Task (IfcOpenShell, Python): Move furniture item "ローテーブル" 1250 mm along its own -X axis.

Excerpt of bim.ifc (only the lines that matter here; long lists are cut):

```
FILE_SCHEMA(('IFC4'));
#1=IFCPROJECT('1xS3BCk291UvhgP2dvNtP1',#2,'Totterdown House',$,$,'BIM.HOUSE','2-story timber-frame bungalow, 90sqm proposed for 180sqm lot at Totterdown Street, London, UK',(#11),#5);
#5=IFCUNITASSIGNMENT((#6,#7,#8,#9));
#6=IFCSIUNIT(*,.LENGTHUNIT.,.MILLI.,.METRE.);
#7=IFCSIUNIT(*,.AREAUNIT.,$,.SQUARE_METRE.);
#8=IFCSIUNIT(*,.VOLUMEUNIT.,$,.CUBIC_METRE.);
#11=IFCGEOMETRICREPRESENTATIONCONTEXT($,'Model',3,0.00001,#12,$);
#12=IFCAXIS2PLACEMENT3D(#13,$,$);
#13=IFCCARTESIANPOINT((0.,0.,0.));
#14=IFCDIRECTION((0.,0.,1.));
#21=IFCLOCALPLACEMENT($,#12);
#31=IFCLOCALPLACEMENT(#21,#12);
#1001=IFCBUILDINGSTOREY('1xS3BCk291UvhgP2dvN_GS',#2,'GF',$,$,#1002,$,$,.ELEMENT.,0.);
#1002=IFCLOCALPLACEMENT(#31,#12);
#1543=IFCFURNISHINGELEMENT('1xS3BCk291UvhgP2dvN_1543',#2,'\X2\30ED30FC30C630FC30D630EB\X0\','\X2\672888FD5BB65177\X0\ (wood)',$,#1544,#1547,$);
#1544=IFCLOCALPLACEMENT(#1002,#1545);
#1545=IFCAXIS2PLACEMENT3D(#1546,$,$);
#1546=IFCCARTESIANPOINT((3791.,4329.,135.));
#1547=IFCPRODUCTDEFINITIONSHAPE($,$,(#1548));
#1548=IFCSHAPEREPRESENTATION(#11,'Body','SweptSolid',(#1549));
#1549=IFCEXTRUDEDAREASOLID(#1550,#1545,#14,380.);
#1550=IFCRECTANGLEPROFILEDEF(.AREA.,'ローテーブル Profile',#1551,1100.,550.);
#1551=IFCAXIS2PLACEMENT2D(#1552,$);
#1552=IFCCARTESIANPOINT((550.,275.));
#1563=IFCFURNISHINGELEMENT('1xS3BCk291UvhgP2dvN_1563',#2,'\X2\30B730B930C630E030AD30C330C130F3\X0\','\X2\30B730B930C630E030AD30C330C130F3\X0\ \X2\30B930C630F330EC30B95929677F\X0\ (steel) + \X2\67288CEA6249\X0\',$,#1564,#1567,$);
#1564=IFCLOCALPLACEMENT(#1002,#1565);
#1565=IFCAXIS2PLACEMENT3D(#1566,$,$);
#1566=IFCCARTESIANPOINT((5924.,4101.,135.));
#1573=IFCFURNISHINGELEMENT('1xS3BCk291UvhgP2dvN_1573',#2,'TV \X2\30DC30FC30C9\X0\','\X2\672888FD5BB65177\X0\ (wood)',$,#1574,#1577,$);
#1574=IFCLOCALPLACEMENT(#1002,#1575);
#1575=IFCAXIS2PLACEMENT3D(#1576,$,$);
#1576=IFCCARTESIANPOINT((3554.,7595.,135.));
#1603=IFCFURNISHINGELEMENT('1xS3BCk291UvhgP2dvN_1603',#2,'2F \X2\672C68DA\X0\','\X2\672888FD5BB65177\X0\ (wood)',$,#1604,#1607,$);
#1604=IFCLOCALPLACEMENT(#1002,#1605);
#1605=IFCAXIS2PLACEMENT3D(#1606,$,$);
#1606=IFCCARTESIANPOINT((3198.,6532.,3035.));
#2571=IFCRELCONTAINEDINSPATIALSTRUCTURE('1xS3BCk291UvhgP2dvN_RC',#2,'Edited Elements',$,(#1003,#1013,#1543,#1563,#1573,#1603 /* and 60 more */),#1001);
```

```python
import ifcopenshell
import ifcopenshell.api.geometry
import ifcopenshell.util.placement
import ifcopenshell.util.unit

model = ifcopenshell.open("bim.ifc")
unit_scale = ifcopenshell.util.unit.calculate_unit_scale(model)

item = model.by_guid("1xS3BCk291UvhgP2dvN_1543")
matrix = ifcopenshell.util.placement.get_local_placement(item.ObjectPlacement)
matrix[:3, 3] -= matrix[:3, 0] * 1.25 / unit_scale
ifcopenshell.api.geometry.edit_object_placement(model, product=item, matrix=matrix, is_si=False)

print(ifcopenshell.util.placement.get_local_placement(item.ObjectPlacement).round(3) + 0.0)

model.write("bim_rev.ifc")
```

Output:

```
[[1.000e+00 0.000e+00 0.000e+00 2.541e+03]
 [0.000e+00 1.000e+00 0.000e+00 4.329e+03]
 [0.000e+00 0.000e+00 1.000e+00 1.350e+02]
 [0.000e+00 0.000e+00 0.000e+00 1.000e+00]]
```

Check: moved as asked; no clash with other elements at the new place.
